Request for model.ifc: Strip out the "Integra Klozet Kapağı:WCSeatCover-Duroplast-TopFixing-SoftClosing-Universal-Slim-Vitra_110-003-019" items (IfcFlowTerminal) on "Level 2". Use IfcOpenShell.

First a look at what the model holds.

```python
import ifcopenshell
import ifcopenshell.util.element

model = ifcopenshell.open("model.ifc")
print(model.schema)
storey = next(s for s in model.by_type("IfcBuildingStorey") if s.Name == "Level 2")
terminals = [e for e in ifcopenshell.util.element.get_decomposition(storey) if e.is_a("IfcFlowTerminal")]
seen = {}
for e in terminals:
    element_type = ifcopenshell.util.element.get_type(e)
    name = element_type.Name if element_type not in (None, e) else None
    seen[name] = seen.get(name, 0) + 1
for name, count in sorted(seen.items(), key=str):
    print(count, "x", name)
```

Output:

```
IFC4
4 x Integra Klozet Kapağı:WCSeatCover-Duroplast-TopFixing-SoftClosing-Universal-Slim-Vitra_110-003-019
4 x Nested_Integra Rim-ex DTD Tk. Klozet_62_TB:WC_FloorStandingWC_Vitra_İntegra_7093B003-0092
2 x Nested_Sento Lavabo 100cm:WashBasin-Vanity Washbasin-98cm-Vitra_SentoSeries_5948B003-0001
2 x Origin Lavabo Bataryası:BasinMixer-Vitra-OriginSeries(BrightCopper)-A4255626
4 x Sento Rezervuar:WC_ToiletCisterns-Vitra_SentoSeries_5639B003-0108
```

```python
import ifcopenshell
import ifcopenshell.api.root
import ifcopenshell.util.element

model = ifcopenshell.open("model.ifc")

storey = next(s for s in model.by_type("IfcBuildingStorey") if s.Name == "Level 2")
terminals = [e for e in ifcopenshell.util.element.get_decomposition(storey) if e.is_a("IfcFlowTerminal")]
targets = [e for e in terminals if (t := ifcopenshell.util.element.get_type(e)) not in (None, e) and t.Name == "Integra Klozet Kapağı:WCSeatCover-Duroplast-TopFixing-SoftClosing-Universal-Slim-Vitra_110-003-019"]

for e in targets:
    ifcopenshell.api.root.remove_product(model, product=e)
print(len(targets), "removed")

model.write("model_rev.ifc")
```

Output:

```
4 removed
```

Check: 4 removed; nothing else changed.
